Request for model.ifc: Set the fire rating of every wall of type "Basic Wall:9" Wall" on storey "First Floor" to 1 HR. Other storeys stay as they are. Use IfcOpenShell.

First a look at what the model holds.

```python
import ifcopenshell
import ifcopenshell.util.element

model = ifcopenshell.open("model.ifc")
print(model.schema)
storey = next(s for s in model.by_type("IfcBuildingStorey") if s.Name == "First Floor")
walls = [e for e in ifcopenshell.util.element.get_decomposition(storey) if e.is_a("IfcWall")]
seen = {}
for e in walls:
    element_type = ifcopenshell.util.element.get_type(e)
    key = (element_type.Name if element_type != e and element_type else None, ifcopenshell.util.element.get_pset(e, "Pset_WallCommon", "FireRating"))
    seen[key] = seen.get(key, 0) + 1
for (name, value), count in sorted(seen.items(), key=str):
    print(count, "x", name, "|", value)
```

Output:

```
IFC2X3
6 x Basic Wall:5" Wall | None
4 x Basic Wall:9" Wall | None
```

```python
import ifcopenshell
import ifcopenshell.api.pset
import ifcopenshell.util.element

model = ifcopenshell.open("model.ifc")

storey = next(s for s in model.by_type("IfcBuildingStorey") if s.Name == "First Floor")
walls = [e for e in ifcopenshell.util.element.get_decomposition(storey) if e.is_a("IfcWall")]

count = 0
for e in walls:
    element_type = ifcopenshell.util.element.get_type(e)
    if element_type in (None, e) or element_type.Name != 'Basic Wall:9" Wall':
        continue
    # add_pset returns the element's existing set when there is one.
    pset = ifcopenshell.api.pset.add_pset(model, product=e, name="Pset_WallCommon")
    ifcopenshell.api.pset.edit_pset(model, pset=pset, properties={"FireRating": "1 HR"})
    count += 1

print(count, "walls updated")

model.write("model_rev.ifc")
```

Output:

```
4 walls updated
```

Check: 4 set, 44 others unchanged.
